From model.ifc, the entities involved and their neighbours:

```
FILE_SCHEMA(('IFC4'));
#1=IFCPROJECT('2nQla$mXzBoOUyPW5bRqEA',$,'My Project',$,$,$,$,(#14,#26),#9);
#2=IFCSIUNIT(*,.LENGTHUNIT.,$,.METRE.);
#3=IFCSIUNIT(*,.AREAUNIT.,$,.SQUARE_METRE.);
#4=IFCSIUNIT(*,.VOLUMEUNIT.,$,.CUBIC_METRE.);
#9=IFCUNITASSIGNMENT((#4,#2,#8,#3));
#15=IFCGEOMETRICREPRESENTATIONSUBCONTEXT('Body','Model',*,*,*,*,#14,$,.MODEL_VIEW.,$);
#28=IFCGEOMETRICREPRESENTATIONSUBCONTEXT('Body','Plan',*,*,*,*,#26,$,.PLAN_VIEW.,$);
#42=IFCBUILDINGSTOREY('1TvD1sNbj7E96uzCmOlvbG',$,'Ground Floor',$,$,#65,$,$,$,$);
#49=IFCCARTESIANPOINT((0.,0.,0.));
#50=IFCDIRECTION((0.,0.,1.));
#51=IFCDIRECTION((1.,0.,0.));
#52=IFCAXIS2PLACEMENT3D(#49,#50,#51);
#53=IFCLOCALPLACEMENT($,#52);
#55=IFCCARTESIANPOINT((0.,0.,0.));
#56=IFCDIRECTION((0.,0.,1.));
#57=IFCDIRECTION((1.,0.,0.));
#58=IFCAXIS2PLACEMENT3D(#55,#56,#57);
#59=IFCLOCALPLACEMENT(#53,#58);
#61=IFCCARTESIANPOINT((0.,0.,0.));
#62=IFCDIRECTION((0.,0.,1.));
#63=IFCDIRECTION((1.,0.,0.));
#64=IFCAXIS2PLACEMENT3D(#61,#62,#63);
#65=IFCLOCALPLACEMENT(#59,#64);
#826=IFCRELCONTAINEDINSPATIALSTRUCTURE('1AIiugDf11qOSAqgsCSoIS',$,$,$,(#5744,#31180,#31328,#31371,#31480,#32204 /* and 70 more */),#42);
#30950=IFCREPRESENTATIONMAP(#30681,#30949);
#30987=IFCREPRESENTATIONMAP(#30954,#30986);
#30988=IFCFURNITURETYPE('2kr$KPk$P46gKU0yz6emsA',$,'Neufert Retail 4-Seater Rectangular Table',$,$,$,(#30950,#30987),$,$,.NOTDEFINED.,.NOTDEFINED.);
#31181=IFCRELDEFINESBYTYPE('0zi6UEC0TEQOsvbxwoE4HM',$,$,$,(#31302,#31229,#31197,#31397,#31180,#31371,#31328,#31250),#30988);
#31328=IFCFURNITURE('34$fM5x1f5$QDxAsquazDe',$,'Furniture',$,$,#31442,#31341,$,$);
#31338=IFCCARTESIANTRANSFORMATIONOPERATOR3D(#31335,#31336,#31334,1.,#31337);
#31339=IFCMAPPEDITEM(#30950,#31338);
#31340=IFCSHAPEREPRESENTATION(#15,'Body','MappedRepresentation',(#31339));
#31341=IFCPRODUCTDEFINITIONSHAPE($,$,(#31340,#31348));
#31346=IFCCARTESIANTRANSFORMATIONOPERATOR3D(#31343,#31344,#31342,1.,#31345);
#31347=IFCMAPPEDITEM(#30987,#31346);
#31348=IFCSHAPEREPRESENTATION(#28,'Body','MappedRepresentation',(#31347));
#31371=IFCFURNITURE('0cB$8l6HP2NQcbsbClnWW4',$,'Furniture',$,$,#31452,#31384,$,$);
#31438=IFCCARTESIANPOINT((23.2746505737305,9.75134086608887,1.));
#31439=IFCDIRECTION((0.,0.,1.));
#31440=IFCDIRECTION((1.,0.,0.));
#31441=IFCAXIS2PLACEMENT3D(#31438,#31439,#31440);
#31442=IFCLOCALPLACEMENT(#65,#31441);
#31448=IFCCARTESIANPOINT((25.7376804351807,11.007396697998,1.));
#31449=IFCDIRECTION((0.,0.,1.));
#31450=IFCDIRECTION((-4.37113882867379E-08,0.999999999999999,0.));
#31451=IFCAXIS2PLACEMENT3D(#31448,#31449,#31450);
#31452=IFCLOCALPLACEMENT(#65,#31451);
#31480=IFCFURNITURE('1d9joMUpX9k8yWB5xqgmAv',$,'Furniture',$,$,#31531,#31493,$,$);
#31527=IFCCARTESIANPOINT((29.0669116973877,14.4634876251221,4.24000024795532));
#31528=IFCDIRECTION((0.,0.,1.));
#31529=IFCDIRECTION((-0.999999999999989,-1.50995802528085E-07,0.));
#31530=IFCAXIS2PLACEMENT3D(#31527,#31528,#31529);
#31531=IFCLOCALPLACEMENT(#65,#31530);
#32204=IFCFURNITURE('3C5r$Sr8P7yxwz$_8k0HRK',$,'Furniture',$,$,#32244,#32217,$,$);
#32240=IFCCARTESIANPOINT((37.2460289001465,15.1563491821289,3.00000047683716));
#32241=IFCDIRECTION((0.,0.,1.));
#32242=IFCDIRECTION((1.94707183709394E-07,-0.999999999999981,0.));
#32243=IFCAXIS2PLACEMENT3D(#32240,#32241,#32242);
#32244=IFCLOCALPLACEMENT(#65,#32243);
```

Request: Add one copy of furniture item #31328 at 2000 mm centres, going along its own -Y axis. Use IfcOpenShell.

```python
import ifcopenshell
import ifcopenshell.api.geometry
import ifcopenshell.api.root
import ifcopenshell.util.element
import ifcopenshell.util.placement
import ifcopenshell.util.unit

model = ifcopenshell.open("model.ifc")
unit_scale = ifcopenshell.util.unit.calculate_unit_scale(model)

source = model.by_guid("34$fM5x1f5$QDxAsquazDe")
base = ifcopenshell.util.placement.get_local_placement(source.ObjectPlacement)
step = -base[:3, 1] * 2 / unit_scale

for i in range(1, 2):
    copy = ifcopenshell.api.root.copy_class(model, product=source)
    copy.Representation = ifcopenshell.util.element.copy_deep(
        model, source.Representation, exclude=["IfcGeometricRepresentationContext", "IfcRepresentationMap"]
    )
    matrix = base.copy()
    matrix[:3, 3] += i * step
    print("added at", matrix[:3, 3].round(3) + 0.0)
    ifcopenshell.api.geometry.edit_object_placement(model, product=copy, matrix=matrix, is_si=False)

model.write("model_v2.ifc")
```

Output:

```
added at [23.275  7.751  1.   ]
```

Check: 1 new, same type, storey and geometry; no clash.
